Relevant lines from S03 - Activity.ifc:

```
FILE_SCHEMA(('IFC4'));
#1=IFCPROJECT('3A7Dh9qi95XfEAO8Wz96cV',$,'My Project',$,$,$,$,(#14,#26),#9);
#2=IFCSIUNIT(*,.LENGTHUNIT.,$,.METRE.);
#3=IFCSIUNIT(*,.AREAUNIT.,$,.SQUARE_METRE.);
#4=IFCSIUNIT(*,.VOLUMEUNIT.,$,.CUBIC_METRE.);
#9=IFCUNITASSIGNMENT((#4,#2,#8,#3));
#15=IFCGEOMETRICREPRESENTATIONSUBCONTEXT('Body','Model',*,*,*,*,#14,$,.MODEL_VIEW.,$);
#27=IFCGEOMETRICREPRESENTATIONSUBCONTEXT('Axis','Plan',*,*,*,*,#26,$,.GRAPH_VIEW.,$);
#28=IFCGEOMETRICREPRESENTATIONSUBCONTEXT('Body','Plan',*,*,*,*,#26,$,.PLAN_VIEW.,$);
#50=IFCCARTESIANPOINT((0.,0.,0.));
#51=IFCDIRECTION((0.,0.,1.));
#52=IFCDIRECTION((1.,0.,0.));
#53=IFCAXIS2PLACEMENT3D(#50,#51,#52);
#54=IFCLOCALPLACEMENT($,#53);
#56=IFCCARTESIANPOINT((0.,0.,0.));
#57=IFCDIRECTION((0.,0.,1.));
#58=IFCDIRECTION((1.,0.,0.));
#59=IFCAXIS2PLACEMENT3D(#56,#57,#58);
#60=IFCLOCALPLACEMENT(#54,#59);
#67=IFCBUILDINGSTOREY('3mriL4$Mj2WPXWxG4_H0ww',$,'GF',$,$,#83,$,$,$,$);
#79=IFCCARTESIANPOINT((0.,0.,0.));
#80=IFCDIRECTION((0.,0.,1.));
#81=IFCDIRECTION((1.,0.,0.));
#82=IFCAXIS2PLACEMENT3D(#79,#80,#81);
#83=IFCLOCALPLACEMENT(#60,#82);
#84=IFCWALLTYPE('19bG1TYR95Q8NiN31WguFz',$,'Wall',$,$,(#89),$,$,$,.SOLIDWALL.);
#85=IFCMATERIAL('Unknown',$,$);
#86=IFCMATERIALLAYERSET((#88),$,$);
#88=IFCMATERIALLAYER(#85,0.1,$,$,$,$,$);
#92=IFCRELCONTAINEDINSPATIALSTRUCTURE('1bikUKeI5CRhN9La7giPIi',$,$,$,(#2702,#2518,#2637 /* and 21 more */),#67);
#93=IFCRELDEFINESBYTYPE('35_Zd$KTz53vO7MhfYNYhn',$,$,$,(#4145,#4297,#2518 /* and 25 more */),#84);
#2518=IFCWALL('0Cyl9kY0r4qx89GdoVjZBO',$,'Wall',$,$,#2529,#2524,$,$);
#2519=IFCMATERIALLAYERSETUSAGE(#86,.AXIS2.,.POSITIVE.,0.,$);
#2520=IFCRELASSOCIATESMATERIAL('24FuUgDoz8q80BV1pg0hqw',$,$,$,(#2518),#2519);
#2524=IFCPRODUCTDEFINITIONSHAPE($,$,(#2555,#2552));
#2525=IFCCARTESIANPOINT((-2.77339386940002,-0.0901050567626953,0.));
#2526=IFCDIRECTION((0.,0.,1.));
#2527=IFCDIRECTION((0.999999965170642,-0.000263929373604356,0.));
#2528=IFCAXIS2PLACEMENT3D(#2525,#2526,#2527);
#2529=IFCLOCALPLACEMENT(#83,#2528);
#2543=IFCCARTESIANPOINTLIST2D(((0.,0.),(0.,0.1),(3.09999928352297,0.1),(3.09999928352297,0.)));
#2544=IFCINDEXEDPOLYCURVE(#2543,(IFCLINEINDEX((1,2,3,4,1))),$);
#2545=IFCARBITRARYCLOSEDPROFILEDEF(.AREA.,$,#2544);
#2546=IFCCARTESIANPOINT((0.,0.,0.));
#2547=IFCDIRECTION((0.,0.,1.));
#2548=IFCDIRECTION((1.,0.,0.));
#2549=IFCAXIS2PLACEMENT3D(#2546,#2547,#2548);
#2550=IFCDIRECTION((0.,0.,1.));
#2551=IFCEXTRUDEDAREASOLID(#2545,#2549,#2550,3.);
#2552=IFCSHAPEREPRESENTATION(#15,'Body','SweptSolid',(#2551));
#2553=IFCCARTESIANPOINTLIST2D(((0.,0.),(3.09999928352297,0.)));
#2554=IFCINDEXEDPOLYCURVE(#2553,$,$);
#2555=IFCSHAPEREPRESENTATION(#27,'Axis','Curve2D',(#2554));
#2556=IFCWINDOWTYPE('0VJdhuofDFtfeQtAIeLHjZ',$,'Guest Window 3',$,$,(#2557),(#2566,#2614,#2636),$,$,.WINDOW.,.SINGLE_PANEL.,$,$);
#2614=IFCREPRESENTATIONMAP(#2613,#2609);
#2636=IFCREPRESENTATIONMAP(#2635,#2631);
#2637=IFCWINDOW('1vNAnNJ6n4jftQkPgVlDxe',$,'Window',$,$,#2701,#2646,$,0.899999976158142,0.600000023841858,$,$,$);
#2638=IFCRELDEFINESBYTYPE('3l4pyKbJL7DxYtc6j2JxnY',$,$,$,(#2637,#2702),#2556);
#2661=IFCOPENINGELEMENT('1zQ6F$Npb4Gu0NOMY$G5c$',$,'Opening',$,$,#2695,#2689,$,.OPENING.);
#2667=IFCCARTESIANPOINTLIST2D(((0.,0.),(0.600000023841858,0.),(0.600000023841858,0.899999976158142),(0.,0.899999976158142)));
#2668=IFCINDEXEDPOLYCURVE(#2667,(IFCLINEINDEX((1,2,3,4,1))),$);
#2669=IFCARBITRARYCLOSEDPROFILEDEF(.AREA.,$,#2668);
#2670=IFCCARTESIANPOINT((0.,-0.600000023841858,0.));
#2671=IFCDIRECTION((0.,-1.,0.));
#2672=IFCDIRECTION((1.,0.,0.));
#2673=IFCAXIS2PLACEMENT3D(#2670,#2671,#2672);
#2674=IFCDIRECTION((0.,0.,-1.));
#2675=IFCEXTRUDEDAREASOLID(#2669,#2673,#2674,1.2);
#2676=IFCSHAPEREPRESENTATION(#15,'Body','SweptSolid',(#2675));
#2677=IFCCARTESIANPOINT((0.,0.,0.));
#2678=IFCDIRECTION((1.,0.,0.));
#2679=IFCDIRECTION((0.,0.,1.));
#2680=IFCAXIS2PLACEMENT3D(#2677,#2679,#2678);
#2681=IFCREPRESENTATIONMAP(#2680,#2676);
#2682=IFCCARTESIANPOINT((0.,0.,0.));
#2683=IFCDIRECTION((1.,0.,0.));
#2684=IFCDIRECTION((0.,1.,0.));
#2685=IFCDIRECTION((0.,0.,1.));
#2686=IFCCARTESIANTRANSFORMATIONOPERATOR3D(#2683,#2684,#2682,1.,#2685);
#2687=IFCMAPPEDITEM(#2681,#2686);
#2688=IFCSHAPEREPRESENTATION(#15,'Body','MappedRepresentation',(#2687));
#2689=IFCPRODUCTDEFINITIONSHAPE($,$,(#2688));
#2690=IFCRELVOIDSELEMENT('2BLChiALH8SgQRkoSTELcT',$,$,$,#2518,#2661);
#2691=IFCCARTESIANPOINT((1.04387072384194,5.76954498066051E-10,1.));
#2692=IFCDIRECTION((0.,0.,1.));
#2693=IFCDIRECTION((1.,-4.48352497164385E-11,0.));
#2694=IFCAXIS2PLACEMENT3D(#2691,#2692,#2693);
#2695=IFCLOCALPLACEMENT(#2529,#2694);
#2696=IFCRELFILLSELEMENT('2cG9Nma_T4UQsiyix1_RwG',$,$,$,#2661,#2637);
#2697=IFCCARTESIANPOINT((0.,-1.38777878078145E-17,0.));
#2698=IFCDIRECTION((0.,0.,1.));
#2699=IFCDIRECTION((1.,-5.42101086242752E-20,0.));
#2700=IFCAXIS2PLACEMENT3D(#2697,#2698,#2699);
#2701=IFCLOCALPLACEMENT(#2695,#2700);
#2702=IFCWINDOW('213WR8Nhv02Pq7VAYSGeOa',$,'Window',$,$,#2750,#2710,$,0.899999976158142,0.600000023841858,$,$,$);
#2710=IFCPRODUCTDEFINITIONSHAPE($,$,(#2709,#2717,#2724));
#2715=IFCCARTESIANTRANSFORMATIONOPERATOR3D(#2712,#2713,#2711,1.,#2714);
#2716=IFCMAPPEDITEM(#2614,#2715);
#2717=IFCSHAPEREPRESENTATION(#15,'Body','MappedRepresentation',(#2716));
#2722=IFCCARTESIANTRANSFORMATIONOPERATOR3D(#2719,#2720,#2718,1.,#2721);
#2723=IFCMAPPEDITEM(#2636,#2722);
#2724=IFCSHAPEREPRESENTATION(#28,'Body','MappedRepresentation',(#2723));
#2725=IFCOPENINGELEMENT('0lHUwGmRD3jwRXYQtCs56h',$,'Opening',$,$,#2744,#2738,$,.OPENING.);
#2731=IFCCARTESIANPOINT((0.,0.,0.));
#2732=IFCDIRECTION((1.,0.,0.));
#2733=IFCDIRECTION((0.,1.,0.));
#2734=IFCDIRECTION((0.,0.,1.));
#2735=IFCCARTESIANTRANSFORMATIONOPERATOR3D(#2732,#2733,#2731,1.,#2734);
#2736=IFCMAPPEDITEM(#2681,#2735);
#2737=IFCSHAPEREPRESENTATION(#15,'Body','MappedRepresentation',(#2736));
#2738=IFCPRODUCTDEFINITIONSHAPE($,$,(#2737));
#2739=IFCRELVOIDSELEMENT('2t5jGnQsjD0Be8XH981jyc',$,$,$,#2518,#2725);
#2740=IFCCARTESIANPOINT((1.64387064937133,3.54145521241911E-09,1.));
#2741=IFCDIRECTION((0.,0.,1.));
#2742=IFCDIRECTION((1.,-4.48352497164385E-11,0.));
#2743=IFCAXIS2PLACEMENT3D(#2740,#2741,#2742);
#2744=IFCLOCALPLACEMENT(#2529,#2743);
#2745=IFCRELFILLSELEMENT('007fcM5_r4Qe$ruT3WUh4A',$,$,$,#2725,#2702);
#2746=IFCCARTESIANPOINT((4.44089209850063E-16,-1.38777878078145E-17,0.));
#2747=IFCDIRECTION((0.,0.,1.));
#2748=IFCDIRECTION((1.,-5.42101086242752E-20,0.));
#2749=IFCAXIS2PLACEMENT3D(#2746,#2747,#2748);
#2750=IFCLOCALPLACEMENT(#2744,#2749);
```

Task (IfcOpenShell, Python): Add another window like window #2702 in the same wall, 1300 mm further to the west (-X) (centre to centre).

```python
import ifcopenshell
import ifcopenshell.api.feature
import ifcopenshell.api.geometry
import ifcopenshell.api.root
import ifcopenshell.geom
import ifcopenshell.util.element
import ifcopenshell.util.placement
import ifcopenshell.util.shape
import ifcopenshell.util.unit

model = ifcopenshell.open("S03 - Activity.ifc")
unit_scale = ifcopenshell.util.unit.calculate_unit_scale(model)
settings = ifcopenshell.geom.settings()


def volume(element):
    """Net volume in cubic metres, openings subtracted."""
    shape = ifcopenshell.geom.create_shape(settings, element)
    return ifcopenshell.util.shape.get_volume(shape.geometry)


window = model.by_guid("213WR8Nhv02Pq7VAYSGeOa")
opening = window.FillsVoids[0].RelatingOpeningElement
wall = opening.VoidsElements[0].RelatingBuildingElement
before = volume(wall)
shift = ifcopenshell.util.placement.get_local_placement(wall.ObjectPlacement)[:3, 0] * -1.3 / unit_scale

# copy_class copies the void relationship, type, container and properties, but no geometry.
new_opening = ifcopenshell.api.root.copy_class(model, product=opening)
new_opening.Representation = ifcopenshell.util.element.copy_deep(
    model, opening.Representation, exclude=["IfcGeometricRepresentationContext", "IfcRepresentationMap"]
)
new_window = ifcopenshell.api.root.copy_class(model, product=window)
new_window.Representation = ifcopenshell.util.element.copy_deep(
    model, window.Representation, exclude=["IfcGeometricRepresentationContext", "IfcRepresentationMap"]
)
ifcopenshell.api.feature.add_filling(model, opening=new_opening, element=new_window)

for old, new in ((opening, new_opening), (window, new_window)):
    matrix = ifcopenshell.util.placement.get_local_placement(old.ObjectPlacement)
    matrix[:3, 3] += shift
    ifcopenshell.api.geometry.edit_object_placement(model, product=new, matrix=matrix, is_si=False)

after = volume(wall)

print(f"wall volume {before:.3f} -> {after:.3f} m3")

model.write("S03 - Activity_updated.ifc")
```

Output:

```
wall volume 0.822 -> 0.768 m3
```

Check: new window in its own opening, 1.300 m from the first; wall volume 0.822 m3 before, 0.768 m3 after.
